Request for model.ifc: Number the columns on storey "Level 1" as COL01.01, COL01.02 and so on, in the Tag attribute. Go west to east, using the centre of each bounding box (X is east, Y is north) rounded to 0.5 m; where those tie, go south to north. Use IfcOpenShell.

First a look at what the model holds.

```python
import ifcopenshell
import ifcopenshell.util.element
import ifcopenshell.util.placement

model = ifcopenshell.open("model.ifc")
print(model.schema)
storey = next(s for s in model.by_type("IfcBuildingStorey") if s.Name == "Level 1")
columns = [e for e in ifcopenshell.util.element.get_decomposition(storey) if e.is_a("IfcColumn")]
for e in sorted(columns, key=lambda e: e.id()):
    origin = ifcopenshell.util.placement.get_local_placement(e.ObjectPlacement)[:3, 3]
    print(e.id(), e.Tag, e.Name, origin.round(2) + 0.0, sep=" | ")
```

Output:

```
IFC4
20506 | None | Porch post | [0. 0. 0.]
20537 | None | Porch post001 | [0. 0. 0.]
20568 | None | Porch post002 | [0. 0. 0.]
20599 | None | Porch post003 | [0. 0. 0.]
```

```python
import ifcopenshell
import ifcopenshell.geom
import ifcopenshell.util.element
import ifcopenshell.util.shape

model = ifcopenshell.open("model.ifc")
settings = ifcopenshell.geom.settings()
settings.set("use-world-coords", True)


def centre(element):
    shape = ifcopenshell.geom.create_shape(settings, element)
    return ifcopenshell.util.shape.get_bbox_centroid(shape.geometry)


storey = next(s for s in model.by_type("IfcBuildingStorey") if s.Name == "Level 1")
columns = [e for e in ifcopenshell.util.element.get_decomposition(storey) if e.is_a("IfcColumn")]

# Insertion points can sit at a corner or the storey origin, so sort by the geometry (in metres).
centres = {e: centre(e) for e in columns}
columns.sort(key=lambda e: (round(centres[e][0] / 0.5), centres[e][1]))

for i, e in enumerate(columns, start=1):
    number = f"COL01.{i:02d}"
    e.Tag = number
    print(e.id(), number)

model.write("model_updated.ifc")
```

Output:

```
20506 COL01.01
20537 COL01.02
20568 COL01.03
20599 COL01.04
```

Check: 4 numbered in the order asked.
